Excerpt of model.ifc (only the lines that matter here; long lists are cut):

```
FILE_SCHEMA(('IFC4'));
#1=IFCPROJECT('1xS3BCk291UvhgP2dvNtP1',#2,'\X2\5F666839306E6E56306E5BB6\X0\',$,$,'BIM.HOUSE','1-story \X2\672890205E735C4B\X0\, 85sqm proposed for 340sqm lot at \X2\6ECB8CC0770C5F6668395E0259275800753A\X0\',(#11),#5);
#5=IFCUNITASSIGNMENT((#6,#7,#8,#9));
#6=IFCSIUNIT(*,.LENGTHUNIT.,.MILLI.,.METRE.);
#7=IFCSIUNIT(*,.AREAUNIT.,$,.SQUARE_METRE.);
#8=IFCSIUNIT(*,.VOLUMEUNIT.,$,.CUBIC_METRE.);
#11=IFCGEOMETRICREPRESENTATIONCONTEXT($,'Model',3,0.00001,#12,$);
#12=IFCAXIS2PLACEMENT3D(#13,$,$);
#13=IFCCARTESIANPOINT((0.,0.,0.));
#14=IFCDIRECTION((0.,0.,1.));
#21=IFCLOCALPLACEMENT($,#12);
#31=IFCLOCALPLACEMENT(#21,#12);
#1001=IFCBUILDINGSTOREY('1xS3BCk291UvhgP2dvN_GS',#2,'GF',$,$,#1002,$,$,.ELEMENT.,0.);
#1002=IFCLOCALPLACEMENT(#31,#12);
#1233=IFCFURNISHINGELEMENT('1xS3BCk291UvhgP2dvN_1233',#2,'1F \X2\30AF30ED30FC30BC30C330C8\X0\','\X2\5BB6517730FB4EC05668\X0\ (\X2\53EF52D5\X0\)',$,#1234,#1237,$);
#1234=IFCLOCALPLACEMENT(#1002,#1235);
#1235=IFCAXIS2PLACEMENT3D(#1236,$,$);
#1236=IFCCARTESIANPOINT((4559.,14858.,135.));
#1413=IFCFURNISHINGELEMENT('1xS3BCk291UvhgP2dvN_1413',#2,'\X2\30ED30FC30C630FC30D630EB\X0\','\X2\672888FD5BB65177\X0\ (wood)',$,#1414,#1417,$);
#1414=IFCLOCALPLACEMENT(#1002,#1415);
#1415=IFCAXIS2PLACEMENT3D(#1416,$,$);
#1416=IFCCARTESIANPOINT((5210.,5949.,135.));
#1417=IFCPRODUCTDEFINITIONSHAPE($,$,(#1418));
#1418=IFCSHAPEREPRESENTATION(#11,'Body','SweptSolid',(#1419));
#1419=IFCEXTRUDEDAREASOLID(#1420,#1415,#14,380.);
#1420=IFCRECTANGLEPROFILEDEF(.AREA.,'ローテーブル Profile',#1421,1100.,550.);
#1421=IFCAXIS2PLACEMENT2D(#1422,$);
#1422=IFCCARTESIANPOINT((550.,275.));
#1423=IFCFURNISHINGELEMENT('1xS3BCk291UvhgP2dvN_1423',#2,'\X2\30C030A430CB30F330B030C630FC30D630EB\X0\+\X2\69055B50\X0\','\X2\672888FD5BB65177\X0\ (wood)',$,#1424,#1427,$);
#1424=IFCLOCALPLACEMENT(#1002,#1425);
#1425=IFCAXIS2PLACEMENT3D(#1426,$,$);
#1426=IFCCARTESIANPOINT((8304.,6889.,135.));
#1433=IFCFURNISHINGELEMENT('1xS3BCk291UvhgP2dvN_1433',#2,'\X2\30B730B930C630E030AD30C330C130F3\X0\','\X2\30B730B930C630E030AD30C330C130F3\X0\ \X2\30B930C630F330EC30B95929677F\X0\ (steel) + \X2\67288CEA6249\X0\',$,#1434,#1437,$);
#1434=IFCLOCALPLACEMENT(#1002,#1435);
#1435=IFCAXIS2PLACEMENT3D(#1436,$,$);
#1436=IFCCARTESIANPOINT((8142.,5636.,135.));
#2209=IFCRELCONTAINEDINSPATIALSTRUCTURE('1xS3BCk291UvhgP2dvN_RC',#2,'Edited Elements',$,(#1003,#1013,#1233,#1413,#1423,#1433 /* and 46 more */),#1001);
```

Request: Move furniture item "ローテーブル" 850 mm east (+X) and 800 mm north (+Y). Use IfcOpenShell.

```python
import ifcopenshell
import ifcopenshell.api.geometry
import ifcopenshell.util.placement
import ifcopenshell.util.unit

model = ifcopenshell.open("model.ifc")
unit_scale = ifcopenshell.util.unit.calculate_unit_scale(model)

item = model.by_guid("1xS3BCk291UvhgP2dvN_1413")
matrix = ifcopenshell.util.placement.get_local_placement(item.ObjectPlacement)
matrix[0, 3] += 0.85 / unit_scale
matrix[1, 3] += 0.8 / unit_scale
ifcopenshell.api.geometry.edit_object_placement(model, product=item, matrix=matrix, is_si=False)

print(ifcopenshell.util.placement.get_local_placement(item.ObjectPlacement).round(3) + 0.0)

model.write("model_v2.ifc")
```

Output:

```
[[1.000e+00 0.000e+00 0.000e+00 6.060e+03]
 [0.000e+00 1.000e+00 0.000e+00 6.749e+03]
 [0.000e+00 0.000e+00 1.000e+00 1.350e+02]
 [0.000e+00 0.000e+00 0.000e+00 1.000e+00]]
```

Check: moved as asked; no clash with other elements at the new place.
